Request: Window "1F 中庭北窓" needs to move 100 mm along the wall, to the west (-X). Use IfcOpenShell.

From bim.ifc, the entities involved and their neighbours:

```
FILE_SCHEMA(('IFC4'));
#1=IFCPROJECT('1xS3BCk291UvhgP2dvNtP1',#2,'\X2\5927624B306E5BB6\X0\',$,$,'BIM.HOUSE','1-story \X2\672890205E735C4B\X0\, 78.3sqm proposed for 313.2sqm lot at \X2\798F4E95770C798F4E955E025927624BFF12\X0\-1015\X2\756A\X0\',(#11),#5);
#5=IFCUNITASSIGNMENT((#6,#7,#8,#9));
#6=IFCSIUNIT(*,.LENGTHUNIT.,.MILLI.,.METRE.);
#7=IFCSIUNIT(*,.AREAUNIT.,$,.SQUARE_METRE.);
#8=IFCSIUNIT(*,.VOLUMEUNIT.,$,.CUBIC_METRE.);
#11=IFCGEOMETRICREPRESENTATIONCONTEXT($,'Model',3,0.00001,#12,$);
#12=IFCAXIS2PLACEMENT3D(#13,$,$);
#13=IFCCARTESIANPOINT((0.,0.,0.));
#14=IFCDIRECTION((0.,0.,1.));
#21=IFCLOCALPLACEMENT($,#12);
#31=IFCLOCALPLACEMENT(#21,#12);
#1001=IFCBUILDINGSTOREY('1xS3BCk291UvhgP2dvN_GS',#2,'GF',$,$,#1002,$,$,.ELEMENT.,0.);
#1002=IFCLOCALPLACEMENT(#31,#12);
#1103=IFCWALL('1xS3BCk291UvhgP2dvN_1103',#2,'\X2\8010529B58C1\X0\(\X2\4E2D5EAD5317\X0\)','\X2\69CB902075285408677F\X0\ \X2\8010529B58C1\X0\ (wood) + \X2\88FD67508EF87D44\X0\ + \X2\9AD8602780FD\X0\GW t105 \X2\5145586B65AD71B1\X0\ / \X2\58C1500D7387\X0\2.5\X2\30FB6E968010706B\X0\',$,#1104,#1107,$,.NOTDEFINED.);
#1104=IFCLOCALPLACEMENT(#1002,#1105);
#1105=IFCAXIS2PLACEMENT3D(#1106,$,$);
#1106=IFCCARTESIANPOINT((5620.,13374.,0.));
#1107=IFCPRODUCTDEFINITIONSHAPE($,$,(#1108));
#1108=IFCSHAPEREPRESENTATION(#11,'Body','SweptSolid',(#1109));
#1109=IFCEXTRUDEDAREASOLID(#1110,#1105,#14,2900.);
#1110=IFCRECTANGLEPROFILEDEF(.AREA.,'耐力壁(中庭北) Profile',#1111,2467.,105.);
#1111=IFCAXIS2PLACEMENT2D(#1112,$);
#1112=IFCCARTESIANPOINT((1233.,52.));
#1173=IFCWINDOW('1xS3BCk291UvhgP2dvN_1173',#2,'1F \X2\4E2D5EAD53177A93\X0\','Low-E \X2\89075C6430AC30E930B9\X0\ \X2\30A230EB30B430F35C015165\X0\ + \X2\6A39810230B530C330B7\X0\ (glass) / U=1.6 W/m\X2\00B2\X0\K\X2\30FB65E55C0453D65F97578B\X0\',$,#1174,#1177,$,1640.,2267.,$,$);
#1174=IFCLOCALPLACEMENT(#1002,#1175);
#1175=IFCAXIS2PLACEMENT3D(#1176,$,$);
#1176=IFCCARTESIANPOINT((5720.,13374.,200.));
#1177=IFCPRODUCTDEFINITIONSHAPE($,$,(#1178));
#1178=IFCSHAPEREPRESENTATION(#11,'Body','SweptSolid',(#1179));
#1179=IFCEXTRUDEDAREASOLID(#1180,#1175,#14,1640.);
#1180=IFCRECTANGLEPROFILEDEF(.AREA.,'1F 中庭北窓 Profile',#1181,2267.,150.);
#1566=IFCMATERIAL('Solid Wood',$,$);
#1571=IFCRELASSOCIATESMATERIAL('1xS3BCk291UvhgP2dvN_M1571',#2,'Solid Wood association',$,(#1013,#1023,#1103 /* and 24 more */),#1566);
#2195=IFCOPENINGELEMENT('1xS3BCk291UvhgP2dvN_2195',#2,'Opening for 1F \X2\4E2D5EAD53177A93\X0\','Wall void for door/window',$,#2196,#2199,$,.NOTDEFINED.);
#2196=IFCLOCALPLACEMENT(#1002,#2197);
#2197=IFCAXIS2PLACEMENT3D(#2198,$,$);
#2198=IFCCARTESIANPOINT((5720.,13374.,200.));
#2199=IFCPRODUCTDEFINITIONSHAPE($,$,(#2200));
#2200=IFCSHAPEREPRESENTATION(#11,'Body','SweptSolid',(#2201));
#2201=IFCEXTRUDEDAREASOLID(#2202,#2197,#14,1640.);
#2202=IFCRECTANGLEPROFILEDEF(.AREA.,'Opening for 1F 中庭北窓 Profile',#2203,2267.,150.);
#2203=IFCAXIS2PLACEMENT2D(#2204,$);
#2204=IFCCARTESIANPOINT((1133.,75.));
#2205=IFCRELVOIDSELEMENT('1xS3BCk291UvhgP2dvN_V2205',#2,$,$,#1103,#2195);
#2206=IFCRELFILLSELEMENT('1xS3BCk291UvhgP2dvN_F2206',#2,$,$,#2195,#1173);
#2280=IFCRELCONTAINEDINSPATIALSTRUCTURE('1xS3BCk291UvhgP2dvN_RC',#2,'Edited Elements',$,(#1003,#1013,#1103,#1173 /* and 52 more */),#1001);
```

```python
import ifcopenshell
import ifcopenshell.api.geometry
import ifcopenshell.util.placement

model = ifcopenshell.open("bim.ifc")

window = model.by_guid("1xS3BCk291UvhgP2dvN_1173")
opening = window.FillsVoids[0].RelatingOpeningElement
wall = opening.VoidsElements[0].RelatingBuildingElement

wall_matrix = ifcopenshell.util.placement.get_local_placement(wall.ObjectPlacement)
shift = wall_matrix[:3, 0] * -100.0
before = ifcopenshell.util.placement.get_local_placement(window.ObjectPlacement)[:3, 3].copy()

# The window is not placed relative to its opening, so move both.
for product in (opening, window):
    matrix = ifcopenshell.util.placement.get_local_placement(product.ObjectPlacement)
    matrix[:3, 3] += shift
    ifcopenshell.api.geometry.edit_object_placement(model, product=product, matrix=matrix, is_si=False)

after = ifcopenshell.util.placement.get_local_placement(window.ObjectPlacement)[:3, 3]
print("window moved by", (after - before).round(3) + 0.0)

model.write("bim-out.ifc")
```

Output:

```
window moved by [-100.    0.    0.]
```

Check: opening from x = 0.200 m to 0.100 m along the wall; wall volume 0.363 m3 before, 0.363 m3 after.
